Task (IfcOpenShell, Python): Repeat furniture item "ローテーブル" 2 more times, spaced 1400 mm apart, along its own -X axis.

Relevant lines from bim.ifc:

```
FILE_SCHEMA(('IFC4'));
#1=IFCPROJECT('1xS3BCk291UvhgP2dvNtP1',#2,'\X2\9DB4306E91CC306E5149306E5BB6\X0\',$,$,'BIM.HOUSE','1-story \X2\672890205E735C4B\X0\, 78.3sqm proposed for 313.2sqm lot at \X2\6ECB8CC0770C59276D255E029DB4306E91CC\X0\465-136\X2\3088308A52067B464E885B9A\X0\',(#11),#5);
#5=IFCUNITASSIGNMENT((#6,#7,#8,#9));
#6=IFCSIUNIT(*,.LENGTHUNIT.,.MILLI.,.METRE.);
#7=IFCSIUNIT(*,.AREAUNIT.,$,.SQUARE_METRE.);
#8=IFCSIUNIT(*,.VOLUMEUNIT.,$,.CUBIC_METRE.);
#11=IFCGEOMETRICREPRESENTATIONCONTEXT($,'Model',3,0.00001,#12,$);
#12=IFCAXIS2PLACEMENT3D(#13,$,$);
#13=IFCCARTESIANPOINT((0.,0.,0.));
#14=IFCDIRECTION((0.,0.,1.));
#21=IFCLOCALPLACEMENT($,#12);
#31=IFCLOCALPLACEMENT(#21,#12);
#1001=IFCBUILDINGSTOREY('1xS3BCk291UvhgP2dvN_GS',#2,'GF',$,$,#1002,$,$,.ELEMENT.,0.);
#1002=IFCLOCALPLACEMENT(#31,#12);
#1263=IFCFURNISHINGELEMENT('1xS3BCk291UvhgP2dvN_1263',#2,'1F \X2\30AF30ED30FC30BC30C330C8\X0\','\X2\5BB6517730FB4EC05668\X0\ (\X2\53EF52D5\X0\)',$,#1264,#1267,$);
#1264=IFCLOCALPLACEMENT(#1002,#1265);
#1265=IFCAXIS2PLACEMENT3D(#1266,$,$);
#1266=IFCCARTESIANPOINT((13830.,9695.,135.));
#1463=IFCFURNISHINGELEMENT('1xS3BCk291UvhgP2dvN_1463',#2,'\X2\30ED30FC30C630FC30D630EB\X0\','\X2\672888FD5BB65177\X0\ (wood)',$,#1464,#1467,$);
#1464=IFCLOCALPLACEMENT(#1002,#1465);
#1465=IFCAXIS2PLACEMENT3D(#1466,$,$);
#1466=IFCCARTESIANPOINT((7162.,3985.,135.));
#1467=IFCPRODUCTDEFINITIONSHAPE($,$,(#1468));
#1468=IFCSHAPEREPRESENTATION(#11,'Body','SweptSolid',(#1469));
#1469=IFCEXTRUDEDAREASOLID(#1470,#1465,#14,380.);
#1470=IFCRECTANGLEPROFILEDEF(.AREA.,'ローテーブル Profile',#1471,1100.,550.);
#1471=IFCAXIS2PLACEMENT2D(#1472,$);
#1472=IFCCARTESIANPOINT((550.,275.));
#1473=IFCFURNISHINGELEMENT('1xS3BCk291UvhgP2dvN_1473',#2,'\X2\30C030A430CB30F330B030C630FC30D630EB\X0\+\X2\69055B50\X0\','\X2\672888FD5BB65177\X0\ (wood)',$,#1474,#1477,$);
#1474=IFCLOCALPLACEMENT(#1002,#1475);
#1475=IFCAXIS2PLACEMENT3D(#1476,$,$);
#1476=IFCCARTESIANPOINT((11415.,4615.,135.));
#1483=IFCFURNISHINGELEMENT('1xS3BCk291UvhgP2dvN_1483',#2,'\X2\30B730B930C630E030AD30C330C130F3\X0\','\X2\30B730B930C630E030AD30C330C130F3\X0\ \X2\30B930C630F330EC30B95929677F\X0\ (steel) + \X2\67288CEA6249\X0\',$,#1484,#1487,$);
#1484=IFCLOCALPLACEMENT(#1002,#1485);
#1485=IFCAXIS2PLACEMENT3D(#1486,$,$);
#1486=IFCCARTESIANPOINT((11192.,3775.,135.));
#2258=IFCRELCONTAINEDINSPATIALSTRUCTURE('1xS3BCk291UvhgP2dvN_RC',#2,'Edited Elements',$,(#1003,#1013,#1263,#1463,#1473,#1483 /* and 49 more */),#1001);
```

```python
import ifcopenshell
import ifcopenshell.api.geometry
import ifcopenshell.api.root
import ifcopenshell.util.element
import ifcopenshell.util.placement

model = ifcopenshell.open("bim.ifc")


def reuse_history(source, copy):
    """copy_class also copies each property set's owner history, people and application; keep the originals."""
    for rel in copy.IsDefinedBy:
        if rel.is_a("IfcRelDefinesByProperties") and (history := rel.RelatingPropertyDefinition.OwnerHistory):
            rel.RelatingPropertyDefinition.OwnerHistory = source.OwnerHistory
            ifcopenshell.util.element.remove_deep2(model, history)


source = model.by_guid("1xS3BCk291UvhgP2dvN_1463")
base = ifcopenshell.util.placement.get_local_placement(source.ObjectPlacement)
step = -base[:3, 0] * 1400.0

for i in range(1, 3):
    copy = ifcopenshell.api.root.copy_class(model, product=source)
    copy.Representation = ifcopenshell.util.element.copy_deep(
        model, source.Representation, exclude=["IfcGeometricRepresentationContext", "IfcRepresentationMap"]
    )
    reuse_history(source, copy)
    matrix = base.copy()
    matrix[:3, 3] += i * step
    print("added at", matrix[:3, 3].round(3) + 0.0)
    ifcopenshell.api.geometry.edit_object_placement(model, product=copy, matrix=matrix, is_si=False)

model.write("bim_rev.ifc")
```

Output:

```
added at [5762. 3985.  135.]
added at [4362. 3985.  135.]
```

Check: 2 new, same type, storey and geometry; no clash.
